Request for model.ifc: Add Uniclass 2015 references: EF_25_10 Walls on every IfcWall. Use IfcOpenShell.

First a look at what the model holds.

```python
import ifcopenshell

model = ifcopenshell.open("model.ifc")
print(model.schema)
print("classifications:", [c.Name for c in model.by_type("IfcClassification")])
for ifc_class in ("IfcDoor", "IfcRoof", "IfcStair", "IfcWall", "IfcWindow"):
    print(ifc_class, len(model.by_type(ifc_class)))
```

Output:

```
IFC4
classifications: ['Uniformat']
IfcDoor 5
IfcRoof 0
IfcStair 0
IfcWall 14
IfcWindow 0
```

```python
import ifcopenshell
import ifcopenshell.api.classification

model = ifcopenshell.open("model.ifc")

system = ifcopenshell.api.classification.add_classification(model, classification="Uniclass 2015")

codes = {
    "IfcWall": ("EF_25_10", "Walls"),
}
for ifc_class, (code, name) in codes.items():
    products = model.by_type(ifc_class)
    ifcopenshell.api.classification.add_reference(
        model, products=products, classification=system, identification=code, name=name
    )
    print(code, len(products))

model.write("model-out.ifc")
```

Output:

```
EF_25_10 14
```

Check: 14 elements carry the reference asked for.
